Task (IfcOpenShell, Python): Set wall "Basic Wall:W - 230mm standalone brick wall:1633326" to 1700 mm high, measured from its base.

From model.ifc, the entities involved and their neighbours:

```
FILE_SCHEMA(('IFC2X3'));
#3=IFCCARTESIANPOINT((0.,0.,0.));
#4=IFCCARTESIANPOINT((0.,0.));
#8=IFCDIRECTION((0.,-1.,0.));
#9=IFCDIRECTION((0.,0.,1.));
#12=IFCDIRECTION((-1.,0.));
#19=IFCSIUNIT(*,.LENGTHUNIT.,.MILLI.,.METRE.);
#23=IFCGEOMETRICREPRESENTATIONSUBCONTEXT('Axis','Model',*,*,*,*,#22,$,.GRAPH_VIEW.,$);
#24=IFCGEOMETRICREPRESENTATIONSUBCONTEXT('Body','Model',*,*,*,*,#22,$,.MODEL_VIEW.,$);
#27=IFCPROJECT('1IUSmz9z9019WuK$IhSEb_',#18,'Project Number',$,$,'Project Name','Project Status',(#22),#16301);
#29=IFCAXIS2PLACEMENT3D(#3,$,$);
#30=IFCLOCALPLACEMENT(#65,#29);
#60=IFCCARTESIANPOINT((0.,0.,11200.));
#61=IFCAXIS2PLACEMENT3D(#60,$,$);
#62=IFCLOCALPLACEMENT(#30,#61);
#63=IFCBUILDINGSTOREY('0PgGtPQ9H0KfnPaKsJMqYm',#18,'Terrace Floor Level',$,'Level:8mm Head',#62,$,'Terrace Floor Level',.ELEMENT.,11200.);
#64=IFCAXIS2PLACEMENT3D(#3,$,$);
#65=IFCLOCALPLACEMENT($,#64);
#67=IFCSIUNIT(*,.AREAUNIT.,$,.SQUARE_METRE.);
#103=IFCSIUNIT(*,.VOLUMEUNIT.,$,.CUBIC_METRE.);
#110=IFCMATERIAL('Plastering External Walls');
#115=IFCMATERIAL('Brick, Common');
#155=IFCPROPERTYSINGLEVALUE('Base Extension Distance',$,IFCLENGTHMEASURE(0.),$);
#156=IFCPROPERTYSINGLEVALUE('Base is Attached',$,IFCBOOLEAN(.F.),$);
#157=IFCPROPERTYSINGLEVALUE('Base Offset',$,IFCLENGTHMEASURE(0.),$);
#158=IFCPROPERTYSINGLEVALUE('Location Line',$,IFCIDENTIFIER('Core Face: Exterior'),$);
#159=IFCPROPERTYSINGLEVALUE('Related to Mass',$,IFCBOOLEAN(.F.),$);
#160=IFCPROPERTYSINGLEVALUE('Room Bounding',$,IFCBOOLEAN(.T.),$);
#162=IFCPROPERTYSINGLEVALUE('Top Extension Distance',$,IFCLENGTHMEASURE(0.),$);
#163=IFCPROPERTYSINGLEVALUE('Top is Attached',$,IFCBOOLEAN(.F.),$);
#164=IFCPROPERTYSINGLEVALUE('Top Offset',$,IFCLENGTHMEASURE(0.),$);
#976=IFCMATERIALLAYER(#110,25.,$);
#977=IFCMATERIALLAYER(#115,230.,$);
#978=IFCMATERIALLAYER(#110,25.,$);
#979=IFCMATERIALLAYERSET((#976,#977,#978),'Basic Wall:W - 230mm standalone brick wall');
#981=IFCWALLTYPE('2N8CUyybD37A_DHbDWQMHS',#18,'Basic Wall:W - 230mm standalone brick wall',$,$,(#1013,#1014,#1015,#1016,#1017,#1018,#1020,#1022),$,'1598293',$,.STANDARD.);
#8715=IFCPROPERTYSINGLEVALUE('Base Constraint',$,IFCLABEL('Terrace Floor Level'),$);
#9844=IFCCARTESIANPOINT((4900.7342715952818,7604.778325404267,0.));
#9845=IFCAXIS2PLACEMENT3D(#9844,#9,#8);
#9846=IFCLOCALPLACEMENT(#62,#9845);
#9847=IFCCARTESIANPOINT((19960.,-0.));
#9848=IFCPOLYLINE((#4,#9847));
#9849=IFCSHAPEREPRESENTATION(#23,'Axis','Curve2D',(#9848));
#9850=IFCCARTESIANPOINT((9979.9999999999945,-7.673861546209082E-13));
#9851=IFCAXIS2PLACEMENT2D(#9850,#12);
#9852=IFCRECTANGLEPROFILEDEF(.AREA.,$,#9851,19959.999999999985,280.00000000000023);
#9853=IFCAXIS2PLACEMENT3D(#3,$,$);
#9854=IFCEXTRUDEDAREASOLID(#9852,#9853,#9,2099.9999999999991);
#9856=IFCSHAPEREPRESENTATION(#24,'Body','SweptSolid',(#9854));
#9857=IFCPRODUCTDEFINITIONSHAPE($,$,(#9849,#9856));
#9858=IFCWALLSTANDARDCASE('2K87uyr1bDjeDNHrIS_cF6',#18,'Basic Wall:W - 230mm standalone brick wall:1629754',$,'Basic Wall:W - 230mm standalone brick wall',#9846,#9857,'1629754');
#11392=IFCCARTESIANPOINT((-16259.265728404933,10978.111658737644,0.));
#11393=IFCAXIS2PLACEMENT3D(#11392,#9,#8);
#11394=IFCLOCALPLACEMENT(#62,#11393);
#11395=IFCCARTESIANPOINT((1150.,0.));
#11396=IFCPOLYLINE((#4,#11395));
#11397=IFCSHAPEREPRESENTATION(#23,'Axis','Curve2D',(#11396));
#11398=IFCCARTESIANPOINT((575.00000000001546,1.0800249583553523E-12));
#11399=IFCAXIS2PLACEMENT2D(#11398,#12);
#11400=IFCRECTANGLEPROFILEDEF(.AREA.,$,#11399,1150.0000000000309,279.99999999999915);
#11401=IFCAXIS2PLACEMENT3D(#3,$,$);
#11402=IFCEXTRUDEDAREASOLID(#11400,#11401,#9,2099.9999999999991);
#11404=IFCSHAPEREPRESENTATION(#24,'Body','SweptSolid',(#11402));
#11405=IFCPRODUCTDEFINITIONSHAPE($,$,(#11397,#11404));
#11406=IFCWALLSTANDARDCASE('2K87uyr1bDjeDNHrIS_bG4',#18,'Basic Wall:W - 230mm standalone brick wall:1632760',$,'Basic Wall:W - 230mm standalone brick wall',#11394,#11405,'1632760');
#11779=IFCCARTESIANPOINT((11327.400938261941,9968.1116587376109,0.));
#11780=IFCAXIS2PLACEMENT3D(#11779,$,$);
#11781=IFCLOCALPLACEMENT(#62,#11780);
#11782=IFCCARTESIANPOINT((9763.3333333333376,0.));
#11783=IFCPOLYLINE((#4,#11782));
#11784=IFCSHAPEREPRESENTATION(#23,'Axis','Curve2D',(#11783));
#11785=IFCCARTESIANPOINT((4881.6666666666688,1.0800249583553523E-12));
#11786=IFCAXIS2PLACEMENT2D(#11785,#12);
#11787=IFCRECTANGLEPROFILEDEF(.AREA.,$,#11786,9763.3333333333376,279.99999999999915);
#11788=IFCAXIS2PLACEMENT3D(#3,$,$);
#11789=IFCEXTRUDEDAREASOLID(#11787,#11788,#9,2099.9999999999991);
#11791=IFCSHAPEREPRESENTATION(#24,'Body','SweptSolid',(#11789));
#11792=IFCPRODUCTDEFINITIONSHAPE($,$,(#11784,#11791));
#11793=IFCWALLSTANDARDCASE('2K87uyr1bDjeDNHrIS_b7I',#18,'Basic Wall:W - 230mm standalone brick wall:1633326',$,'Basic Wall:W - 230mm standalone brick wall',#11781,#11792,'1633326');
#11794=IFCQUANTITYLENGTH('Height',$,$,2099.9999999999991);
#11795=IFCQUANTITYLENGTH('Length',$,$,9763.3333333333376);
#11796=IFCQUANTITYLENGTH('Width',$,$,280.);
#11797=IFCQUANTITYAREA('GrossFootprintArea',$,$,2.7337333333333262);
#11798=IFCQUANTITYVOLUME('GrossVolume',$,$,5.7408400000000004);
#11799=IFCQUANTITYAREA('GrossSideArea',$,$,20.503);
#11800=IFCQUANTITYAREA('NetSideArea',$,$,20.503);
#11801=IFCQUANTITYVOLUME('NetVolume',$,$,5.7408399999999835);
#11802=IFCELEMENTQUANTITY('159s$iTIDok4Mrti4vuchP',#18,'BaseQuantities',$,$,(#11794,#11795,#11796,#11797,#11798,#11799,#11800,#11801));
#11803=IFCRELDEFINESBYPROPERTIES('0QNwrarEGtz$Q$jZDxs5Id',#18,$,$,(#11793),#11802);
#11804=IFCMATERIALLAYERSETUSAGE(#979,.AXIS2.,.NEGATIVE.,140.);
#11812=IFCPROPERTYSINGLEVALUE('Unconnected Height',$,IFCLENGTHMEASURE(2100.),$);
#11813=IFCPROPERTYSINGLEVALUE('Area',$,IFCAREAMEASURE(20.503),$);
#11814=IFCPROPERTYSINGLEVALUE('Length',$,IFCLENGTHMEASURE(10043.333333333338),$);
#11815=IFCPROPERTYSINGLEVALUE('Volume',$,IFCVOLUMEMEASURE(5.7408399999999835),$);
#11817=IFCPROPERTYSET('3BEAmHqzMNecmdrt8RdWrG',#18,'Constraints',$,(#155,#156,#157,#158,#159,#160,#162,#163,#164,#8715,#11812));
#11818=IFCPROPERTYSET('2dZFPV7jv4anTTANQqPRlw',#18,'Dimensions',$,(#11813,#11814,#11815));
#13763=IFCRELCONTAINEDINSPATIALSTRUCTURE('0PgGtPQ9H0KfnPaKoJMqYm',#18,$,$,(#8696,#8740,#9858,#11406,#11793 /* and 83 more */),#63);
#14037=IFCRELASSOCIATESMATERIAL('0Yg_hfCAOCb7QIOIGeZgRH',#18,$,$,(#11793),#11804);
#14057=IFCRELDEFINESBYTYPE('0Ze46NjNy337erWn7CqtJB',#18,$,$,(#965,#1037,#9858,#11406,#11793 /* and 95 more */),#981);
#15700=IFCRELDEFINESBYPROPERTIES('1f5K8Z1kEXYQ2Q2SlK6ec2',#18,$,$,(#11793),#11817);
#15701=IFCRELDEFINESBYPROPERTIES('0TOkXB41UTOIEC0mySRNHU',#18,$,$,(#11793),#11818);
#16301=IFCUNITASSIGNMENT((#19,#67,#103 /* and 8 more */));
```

```python
import ifcopenshell
import ifcopenshell.api.pset
import ifcopenshell.geom
import ifcopenshell.util.element
import ifcopenshell.util.representation
import ifcopenshell.util.shape
import ifcopenshell.util.unit

model = ifcopenshell.open("model.ifc")
unit_scale = ifcopenshell.util.unit.calculate_unit_scale(model)
area_scale = ifcopenshell.util.unit.calculate_unit_scale(model, "AREAUNIT")
volume_scale = ifcopenshell.util.unit.calculate_unit_scale(model, "VOLUMEUNIT")
settings = ifcopenshell.geom.settings()


def volume(element):
    """Net volume in cubic metres, openings subtracted."""
    shape = ifcopenshell.geom.create_shape(settings, element)
    return ifcopenshell.util.shape.get_volume(shape.geometry)


wall = model.by_guid("2K87uyr1bDjeDNHrIS_b7I")
before = volume(wall)

body = ifcopenshell.util.representation.get_representation(wall, "Model", "Body")
solid = body.Items[0]
old_height = solid.Depth
solid.Depth = 1.7 / unit_scale
after = volume(wall)
thickness = 0.28  # wall thickness in metres

# Update the stored height, areas and volumes.
qto = model.by_id(ifcopenshell.util.element.get_pset(wall, "BaseQuantities", should_inherit=False)["id"])
ifcopenshell.api.pset.edit_qto(model, qto=qto, properties={
    "Height": solid.Depth,
    "GrossVolume": ifcopenshell.util.element.get_pset(wall, "BaseQuantities", "GrossVolume") * solid.Depth / old_height,
    "GrossSideArea": ifcopenshell.util.element.get_pset(wall, "BaseQuantities", "GrossSideArea") * solid.Depth / old_height,
    "NetSideArea": after / thickness / area_scale,
    "NetVolume": after / volume_scale,
})
pset = model.by_id(ifcopenshell.util.element.get_pset(wall, "Constraints", should_inherit=False)["id"])
ifcopenshell.api.pset.edit_pset(model, pset=pset, properties={
    "Unconnected Height": model.create_entity("IfcLengthMeasure", solid.Depth),
})
pset = model.by_id(ifcopenshell.util.element.get_pset(wall, "Dimensions", should_inherit=False)["id"])
ifcopenshell.api.pset.edit_pset(model, pset=pset, properties={
    "Area": model.create_entity("IfcAreaMeasure", after / thickness / area_scale),
    "Volume": model.create_entity("IfcVolumeMeasure", after / volume_scale),
})

print(f"height {old_height:g} -> {solid.Depth:g}, volume {before:.3f} -> {after:.3f} m3")

model.write("model_updated.ifc")
```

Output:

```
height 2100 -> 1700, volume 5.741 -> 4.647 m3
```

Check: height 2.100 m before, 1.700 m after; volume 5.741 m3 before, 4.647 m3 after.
